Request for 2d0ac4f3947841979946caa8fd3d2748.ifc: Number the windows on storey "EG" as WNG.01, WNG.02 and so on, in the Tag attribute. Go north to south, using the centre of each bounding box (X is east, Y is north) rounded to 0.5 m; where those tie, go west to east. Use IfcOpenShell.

First a look at what the model holds.

```python
import ifcopenshell
import ifcopenshell.util.element
import ifcopenshell.util.placement

model = ifcopenshell.open("2d0ac4f3947841979946caa8fd3d2748.ifc")
print(model.schema)
storey = next(s for s in model.by_type("IfcBuildingStorey") if s.Name == "EG")
windows = [e for e in ifcopenshell.util.element.get_decomposition(storey) if e.is_a("IfcWindow")]
for e in sorted(windows, key=lambda e: e.id()):
    origin = ifcopenshell.util.placement.get_local_placement(e.ObjectPlacement)[:3, 3]
    print(e.id(), e.Tag, e.Name, origin.round(2) + 0.0, sep=" | ")
```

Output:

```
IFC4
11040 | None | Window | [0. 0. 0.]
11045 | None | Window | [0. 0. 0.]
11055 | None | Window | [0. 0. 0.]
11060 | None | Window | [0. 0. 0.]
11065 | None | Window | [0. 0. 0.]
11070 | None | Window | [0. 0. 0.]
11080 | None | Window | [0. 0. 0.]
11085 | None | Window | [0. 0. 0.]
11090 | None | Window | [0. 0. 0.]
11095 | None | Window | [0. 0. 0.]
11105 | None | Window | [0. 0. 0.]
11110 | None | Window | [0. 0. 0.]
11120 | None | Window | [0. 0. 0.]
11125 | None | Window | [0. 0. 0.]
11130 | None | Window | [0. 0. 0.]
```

```python
import ifcopenshell
import ifcopenshell.geom
import ifcopenshell.util.element
import ifcopenshell.util.shape

model = ifcopenshell.open("2d0ac4f3947841979946caa8fd3d2748.ifc")
settings = ifcopenshell.geom.settings()
settings.set("use-world-coords", True)


def centre(element):
    shape = ifcopenshell.geom.create_shape(settings, element)
    return ifcopenshell.util.shape.get_bbox_centroid(shape.geometry)


storey = next(s for s in model.by_type("IfcBuildingStorey") if s.Name == "EG")
windows = [e for e in ifcopenshell.util.element.get_decomposition(storey) if e.is_a("IfcWindow")]

# Insertion points can sit at a corner or the storey origin, so sort by the geometry (in metres).
centres = {e: centre(e) for e in windows}
windows.sort(key=lambda e: (-round(centres[e][1] / 0.5), centres[e][0]))

for i, e in enumerate(windows, start=1):
    number = f"WNG.{i:02d}"
    e.Tag = number
    print(e.id(), number)

model.write("2d0ac4f3947841979946caa8fd3d2748_v2.ifc")
```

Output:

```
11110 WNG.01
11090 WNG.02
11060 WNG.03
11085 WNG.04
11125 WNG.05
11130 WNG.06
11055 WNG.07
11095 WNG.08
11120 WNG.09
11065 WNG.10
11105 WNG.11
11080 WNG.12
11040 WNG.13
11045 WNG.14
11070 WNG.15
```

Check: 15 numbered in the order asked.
